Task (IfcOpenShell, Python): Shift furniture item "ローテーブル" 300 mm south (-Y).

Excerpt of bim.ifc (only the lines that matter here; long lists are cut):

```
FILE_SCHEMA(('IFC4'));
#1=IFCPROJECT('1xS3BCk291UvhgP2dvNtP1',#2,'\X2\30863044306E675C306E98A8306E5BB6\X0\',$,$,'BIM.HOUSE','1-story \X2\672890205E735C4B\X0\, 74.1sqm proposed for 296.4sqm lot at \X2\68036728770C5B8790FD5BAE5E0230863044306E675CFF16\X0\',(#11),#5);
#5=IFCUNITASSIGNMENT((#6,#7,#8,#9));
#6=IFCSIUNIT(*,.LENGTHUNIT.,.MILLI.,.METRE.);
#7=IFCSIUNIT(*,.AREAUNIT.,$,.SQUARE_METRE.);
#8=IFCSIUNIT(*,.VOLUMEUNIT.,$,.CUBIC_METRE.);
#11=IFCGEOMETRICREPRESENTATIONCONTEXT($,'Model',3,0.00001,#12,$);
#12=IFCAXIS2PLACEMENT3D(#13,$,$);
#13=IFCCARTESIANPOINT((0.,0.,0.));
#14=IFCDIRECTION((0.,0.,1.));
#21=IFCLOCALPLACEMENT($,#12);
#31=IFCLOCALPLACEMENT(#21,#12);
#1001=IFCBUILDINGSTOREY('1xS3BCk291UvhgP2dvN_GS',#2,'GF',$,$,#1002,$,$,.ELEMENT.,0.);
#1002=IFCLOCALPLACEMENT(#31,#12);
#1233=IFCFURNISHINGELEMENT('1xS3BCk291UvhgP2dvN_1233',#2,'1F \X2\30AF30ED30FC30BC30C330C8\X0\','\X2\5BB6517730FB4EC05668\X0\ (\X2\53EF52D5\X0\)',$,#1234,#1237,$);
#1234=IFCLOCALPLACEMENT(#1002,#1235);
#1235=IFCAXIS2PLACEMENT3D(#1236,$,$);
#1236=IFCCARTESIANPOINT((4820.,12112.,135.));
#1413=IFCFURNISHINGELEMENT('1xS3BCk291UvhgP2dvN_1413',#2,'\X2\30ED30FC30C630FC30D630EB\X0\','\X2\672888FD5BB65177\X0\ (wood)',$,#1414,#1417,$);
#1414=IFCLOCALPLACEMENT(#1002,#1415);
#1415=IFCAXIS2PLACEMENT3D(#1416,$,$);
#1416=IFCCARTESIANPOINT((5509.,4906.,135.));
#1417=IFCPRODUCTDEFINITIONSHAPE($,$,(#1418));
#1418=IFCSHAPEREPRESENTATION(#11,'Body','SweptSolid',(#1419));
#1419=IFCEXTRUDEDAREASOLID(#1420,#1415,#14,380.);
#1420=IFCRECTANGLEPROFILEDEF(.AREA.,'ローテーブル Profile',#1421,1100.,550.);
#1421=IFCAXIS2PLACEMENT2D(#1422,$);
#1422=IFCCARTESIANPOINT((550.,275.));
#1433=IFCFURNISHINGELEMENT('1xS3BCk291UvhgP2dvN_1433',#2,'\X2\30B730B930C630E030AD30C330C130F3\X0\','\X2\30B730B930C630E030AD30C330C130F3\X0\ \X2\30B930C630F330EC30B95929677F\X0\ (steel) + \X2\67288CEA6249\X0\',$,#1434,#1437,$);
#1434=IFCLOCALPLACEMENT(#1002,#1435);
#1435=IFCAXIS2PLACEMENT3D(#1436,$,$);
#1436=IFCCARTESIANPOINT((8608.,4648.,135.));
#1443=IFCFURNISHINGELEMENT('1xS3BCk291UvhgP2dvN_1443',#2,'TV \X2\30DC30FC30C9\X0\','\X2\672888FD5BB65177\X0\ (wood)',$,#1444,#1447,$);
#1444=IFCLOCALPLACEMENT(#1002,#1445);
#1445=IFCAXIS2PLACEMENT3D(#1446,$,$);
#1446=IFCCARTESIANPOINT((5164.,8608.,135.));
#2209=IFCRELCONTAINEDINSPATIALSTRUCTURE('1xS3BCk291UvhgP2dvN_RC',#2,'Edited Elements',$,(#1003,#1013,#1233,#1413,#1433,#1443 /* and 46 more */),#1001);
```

```python
import ifcopenshell
import ifcopenshell.api.geometry
import ifcopenshell.util.placement
import ifcopenshell.util.unit

model = ifcopenshell.open("bim.ifc")
unit_scale = ifcopenshell.util.unit.calculate_unit_scale(model)

item = model.by_guid("1xS3BCk291UvhgP2dvN_1413")
matrix = ifcopenshell.util.placement.get_local_placement(item.ObjectPlacement)
matrix[1, 3] -= 0.3 / unit_scale
ifcopenshell.api.geometry.edit_object_placement(model, product=item, matrix=matrix, is_si=False)

print(ifcopenshell.util.placement.get_local_placement(item.ObjectPlacement).round(3) + 0.0)

model.write("bim_edited.ifc")
```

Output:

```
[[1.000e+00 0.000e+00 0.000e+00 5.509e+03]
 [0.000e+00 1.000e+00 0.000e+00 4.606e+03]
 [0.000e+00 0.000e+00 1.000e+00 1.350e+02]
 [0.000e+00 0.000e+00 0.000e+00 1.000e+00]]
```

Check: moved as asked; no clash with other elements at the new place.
